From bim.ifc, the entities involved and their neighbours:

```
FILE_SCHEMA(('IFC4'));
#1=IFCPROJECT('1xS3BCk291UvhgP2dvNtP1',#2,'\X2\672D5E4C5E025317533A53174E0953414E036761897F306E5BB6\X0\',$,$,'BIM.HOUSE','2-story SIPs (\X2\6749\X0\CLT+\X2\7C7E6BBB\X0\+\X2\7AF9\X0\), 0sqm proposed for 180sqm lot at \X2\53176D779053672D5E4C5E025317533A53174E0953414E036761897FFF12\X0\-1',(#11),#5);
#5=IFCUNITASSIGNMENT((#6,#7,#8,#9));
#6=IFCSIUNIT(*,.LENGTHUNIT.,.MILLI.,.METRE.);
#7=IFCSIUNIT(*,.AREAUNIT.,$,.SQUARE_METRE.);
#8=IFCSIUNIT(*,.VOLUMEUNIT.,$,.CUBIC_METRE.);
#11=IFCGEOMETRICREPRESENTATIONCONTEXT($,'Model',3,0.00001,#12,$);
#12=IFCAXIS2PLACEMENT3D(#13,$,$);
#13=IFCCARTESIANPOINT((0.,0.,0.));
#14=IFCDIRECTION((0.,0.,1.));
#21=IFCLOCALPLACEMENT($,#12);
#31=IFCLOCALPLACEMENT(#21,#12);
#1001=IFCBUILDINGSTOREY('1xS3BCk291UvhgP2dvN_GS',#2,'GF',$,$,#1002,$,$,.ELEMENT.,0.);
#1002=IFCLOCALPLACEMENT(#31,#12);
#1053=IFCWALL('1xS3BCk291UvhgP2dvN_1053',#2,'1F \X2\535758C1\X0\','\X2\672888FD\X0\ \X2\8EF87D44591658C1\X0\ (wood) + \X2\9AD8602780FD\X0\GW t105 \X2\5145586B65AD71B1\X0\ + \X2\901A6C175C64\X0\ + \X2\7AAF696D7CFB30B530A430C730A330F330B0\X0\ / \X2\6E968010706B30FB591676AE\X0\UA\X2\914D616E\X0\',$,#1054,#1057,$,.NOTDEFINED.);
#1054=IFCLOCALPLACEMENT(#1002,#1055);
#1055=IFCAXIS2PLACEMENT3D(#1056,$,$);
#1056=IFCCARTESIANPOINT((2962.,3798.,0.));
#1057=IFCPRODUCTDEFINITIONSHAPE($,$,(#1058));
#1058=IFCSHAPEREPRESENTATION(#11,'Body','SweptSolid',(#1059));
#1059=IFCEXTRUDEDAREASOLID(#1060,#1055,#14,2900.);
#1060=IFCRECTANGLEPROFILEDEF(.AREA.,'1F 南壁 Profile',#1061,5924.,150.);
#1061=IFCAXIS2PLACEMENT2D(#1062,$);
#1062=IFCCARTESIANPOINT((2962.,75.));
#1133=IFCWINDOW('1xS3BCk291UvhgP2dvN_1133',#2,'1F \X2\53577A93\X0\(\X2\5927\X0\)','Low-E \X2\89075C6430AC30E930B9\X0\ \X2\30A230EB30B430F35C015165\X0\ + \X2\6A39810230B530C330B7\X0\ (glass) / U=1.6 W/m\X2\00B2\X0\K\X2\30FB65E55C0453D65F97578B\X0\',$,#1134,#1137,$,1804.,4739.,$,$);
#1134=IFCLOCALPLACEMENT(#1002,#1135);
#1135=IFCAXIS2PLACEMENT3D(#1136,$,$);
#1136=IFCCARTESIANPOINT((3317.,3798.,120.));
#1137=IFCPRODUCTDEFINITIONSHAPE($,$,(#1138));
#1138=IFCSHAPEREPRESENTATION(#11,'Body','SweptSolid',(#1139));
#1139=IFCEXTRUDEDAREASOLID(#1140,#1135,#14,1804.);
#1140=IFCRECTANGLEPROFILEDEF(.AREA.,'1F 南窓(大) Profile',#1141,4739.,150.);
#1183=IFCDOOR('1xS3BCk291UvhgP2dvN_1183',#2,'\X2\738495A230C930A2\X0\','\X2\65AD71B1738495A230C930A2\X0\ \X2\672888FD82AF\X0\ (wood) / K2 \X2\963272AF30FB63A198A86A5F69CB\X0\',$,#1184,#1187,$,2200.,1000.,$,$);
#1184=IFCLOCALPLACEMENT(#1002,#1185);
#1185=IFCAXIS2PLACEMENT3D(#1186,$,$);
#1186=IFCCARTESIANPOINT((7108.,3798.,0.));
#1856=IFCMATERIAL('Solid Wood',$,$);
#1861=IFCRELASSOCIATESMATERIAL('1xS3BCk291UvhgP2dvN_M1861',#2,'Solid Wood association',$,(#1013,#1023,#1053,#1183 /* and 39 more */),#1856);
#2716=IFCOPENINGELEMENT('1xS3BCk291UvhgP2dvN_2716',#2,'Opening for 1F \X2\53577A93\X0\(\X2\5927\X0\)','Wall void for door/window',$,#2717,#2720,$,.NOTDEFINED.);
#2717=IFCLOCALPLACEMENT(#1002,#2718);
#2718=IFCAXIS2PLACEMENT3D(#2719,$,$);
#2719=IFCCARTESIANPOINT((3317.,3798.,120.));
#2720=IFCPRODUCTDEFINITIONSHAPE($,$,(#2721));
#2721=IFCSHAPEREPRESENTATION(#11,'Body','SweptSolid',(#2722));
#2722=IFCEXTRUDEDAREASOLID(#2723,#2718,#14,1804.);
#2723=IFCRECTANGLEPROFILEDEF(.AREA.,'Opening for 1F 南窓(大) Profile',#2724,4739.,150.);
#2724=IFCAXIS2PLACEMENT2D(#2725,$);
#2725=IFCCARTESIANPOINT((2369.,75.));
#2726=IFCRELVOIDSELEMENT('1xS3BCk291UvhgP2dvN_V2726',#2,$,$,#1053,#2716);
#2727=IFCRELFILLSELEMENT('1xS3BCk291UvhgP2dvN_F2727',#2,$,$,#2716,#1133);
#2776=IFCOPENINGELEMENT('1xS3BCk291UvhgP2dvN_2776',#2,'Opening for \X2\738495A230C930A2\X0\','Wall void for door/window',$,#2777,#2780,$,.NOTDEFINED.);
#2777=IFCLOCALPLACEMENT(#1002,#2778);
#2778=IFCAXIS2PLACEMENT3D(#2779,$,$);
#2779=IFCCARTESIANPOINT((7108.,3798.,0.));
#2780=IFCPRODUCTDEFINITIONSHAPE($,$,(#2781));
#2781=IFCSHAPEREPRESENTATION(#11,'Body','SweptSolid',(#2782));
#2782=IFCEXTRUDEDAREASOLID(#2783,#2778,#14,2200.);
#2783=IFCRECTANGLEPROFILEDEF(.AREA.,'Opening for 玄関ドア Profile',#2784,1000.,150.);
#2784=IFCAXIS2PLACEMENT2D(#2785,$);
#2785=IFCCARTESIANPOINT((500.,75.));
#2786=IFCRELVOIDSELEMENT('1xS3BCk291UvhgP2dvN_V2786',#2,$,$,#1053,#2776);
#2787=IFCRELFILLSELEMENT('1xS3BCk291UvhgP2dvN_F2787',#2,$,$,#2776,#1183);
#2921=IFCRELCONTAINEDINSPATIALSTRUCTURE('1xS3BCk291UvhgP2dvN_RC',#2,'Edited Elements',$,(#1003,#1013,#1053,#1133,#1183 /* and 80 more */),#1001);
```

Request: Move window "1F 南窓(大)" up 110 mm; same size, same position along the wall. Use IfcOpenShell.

```python
import numpy as np
import ifcopenshell
import ifcopenshell.api.geometry
import ifcopenshell.util.placement
import ifcopenshell.util.unit

model = ifcopenshell.open("bim.ifc")
unit_scale = ifcopenshell.util.unit.calculate_unit_scale(model)

window = model.by_guid("1xS3BCk291UvhgP2dvN_1133")
opening = window.FillsVoids[0].RelatingOpeningElement
dz = 0.11 / unit_scale

shift = np.array([0.0, 0.0, dz])
# The window is not placed relative to its opening, so move both.
for product in (opening, window):
    matrix = ifcopenshell.util.placement.get_local_placement(product.ObjectPlacement)
    matrix[:3, 3] += shift
    ifcopenshell.api.geometry.edit_object_placement(model, product=product, matrix=matrix, is_si=False)

print(f"moved by {dz * unit_scale:+.3f} m")

model.write("bim_rev.ifc")
```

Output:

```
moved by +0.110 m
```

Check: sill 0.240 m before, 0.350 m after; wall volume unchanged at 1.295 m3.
